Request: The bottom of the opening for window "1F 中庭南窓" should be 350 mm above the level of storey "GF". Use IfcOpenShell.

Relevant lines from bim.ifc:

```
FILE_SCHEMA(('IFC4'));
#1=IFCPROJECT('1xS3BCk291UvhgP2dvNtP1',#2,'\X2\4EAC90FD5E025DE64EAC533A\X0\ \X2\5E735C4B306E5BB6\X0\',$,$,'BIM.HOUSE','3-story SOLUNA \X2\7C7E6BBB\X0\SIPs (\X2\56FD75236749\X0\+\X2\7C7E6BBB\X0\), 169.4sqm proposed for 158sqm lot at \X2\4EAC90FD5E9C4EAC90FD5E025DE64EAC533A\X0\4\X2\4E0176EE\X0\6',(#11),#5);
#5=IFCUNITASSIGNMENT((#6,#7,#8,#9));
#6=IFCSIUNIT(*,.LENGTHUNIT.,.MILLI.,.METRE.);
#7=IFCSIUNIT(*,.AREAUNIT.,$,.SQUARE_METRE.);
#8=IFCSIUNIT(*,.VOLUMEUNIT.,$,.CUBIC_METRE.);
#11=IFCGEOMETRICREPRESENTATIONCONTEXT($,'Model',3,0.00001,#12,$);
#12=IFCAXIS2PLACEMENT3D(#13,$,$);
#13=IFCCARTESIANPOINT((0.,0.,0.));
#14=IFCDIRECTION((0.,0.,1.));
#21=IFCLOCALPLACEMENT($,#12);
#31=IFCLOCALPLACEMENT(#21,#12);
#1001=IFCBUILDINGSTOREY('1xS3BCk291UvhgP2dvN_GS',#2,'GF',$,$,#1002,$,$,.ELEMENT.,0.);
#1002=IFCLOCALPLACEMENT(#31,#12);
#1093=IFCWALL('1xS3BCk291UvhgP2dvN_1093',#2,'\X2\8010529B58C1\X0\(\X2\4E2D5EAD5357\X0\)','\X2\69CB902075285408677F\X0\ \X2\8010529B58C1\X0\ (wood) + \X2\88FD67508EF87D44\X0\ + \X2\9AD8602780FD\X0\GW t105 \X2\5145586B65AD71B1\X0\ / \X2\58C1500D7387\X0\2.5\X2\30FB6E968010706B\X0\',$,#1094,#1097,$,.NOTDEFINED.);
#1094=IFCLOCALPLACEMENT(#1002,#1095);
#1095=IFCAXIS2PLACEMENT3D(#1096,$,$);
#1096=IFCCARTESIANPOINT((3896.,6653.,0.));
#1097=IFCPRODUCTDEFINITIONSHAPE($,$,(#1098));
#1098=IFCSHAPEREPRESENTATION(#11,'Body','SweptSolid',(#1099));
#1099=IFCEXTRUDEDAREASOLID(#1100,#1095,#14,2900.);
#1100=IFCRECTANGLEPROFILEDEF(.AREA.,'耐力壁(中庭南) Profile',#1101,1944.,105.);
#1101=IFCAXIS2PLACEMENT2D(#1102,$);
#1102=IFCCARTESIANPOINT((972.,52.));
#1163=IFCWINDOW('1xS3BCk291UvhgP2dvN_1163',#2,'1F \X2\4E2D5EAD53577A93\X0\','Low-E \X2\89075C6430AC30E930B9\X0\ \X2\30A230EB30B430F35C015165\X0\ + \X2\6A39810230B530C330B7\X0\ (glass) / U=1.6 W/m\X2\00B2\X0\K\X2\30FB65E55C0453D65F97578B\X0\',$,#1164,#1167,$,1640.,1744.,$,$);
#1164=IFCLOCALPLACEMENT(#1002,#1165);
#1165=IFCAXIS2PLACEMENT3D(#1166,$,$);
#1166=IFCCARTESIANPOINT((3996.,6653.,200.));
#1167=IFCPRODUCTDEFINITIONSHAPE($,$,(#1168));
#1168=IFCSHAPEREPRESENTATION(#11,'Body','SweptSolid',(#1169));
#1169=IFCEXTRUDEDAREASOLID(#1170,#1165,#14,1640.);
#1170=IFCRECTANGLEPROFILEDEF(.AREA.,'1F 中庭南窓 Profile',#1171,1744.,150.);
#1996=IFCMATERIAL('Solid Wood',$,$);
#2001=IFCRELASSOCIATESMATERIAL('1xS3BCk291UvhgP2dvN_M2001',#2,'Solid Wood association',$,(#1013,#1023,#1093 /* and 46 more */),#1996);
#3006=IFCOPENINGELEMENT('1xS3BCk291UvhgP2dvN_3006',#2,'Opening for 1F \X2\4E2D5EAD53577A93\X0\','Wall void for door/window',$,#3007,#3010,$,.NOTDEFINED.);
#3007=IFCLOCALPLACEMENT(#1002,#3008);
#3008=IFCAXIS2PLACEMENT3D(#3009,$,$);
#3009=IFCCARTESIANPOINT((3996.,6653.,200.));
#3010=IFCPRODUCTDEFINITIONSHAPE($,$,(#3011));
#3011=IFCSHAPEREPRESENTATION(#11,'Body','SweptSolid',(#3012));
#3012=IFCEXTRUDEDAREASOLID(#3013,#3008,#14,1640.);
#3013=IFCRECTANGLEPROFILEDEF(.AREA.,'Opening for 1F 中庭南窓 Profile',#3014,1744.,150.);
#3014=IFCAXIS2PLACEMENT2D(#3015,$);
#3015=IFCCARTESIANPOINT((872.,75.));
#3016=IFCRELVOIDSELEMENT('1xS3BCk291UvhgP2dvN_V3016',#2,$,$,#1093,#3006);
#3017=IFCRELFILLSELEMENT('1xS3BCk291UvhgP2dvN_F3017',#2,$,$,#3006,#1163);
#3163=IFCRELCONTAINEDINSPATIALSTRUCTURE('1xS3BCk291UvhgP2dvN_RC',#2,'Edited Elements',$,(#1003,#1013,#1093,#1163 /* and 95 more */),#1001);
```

```python
import numpy as np
import ifcopenshell
import ifcopenshell.api.geometry
import ifcopenshell.geom
import ifcopenshell.util.element
import ifcopenshell.util.placement
import ifcopenshell.util.shape
import ifcopenshell.util.unit

model = ifcopenshell.open("bim.ifc")
unit_scale = ifcopenshell.util.unit.calculate_unit_scale(model)

window = model.by_id(1163)
opening = window.FillsVoids[0].RelatingOpeningElement
storey = ifcopenshell.util.element.get_container(window, ifc_class="IfcBuildingStorey")
level = ifcopenshell.util.placement.get_local_placement(storey.ObjectPlacement)[2, 3]

# The opening's origin need not be at the sill, so measure its lowest point.
shape = ifcopenshell.geom.create_shape(ifcopenshell.geom.settings(), opening)
bottom = ifcopenshell.util.shape.get_shape_bottom_elevation(shape, shape.geometry) / unit_scale
dz = level + 0.35 / unit_scale - bottom

shift = np.array([0.0, 0.0, dz])
# The window is not placed relative to its opening, so move both.
for product in (opening, window):
    matrix = ifcopenshell.util.placement.get_local_placement(product.ObjectPlacement)
    matrix[:3, 3] += shift
    ifcopenshell.api.geometry.edit_object_placement(model, product=product, matrix=matrix, is_si=False)

print(f"moved by {dz * unit_scale:+.3f} m")

model.write("bim_edited.ifc")
```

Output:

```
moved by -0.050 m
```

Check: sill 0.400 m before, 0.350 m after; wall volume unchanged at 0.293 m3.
